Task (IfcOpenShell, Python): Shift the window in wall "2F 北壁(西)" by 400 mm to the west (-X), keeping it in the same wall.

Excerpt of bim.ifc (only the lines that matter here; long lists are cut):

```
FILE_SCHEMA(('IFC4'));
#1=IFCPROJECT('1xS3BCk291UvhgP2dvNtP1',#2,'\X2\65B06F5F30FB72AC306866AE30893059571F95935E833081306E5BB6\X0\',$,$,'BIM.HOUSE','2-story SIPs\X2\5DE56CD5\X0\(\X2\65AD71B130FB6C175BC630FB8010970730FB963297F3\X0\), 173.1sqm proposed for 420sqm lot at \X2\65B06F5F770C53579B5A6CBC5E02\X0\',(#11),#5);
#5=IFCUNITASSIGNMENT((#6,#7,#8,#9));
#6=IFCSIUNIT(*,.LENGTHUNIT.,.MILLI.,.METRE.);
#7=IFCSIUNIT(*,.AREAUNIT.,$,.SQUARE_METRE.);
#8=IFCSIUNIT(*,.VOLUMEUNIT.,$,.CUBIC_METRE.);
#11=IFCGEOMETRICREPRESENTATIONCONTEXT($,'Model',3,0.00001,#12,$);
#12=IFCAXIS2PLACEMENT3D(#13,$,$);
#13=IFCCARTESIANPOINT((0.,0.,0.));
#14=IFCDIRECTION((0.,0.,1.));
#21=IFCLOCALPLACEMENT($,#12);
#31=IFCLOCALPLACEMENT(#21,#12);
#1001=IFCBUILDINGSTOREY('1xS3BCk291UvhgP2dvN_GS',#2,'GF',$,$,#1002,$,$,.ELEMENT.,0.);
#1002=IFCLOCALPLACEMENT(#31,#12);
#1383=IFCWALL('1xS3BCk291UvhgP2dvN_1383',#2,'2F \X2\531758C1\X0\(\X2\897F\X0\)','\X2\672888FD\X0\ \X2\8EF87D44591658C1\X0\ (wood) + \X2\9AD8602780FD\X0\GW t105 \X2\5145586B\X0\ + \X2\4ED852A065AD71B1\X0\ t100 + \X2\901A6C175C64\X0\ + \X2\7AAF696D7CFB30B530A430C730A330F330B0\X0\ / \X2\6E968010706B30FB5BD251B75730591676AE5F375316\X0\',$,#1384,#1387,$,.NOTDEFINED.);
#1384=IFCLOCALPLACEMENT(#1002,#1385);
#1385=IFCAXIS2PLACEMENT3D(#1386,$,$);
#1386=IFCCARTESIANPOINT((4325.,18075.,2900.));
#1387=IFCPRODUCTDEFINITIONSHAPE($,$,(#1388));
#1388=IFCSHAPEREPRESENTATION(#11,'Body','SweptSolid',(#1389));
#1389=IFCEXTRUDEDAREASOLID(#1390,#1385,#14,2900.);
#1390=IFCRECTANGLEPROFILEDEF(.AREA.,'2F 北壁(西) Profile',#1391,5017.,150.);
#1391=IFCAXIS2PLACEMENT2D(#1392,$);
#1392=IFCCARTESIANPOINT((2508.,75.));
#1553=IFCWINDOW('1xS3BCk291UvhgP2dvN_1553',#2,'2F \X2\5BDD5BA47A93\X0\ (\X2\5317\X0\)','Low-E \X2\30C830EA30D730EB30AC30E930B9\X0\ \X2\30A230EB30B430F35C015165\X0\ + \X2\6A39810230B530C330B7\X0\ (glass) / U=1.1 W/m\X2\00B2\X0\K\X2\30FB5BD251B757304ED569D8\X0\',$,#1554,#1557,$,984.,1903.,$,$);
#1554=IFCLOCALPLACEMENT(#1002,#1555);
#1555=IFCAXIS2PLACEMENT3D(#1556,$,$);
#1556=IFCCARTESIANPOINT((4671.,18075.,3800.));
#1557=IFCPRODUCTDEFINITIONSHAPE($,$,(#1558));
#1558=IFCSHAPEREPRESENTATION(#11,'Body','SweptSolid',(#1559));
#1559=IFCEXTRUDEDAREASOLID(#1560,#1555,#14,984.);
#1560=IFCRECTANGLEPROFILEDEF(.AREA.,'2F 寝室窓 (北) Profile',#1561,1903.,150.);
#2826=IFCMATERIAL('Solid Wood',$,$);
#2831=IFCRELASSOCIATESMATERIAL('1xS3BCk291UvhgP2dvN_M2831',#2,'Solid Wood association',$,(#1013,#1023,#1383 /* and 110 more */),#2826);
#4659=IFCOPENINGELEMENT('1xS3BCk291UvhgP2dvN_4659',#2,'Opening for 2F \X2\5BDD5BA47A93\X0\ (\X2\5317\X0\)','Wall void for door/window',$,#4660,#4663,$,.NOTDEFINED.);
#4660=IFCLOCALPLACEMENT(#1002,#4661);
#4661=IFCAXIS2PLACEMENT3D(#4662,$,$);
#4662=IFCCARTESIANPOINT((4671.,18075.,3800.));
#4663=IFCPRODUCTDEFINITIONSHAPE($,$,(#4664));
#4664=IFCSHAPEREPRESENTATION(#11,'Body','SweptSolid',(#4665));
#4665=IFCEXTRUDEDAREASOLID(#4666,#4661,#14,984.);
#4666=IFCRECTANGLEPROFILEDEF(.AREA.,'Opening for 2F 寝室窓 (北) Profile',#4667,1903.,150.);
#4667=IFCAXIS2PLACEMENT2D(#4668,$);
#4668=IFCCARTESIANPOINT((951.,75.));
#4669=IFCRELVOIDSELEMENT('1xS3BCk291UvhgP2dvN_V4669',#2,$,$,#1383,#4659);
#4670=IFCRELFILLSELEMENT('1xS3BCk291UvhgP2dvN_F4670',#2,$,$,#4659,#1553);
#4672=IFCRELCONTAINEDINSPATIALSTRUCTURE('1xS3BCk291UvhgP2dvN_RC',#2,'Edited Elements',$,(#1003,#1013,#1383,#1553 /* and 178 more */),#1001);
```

```python
import ifcopenshell
import ifcopenshell.api.geometry
import ifcopenshell.util.placement

model = ifcopenshell.open("bim.ifc")

window = model.by_id(1553)
opening = window.FillsVoids[0].RelatingOpeningElement
wall = opening.VoidsElements[0].RelatingBuildingElement

wall_matrix = ifcopenshell.util.placement.get_local_placement(wall.ObjectPlacement)
shift = wall_matrix[:3, 0] * -400.0
before = ifcopenshell.util.placement.get_local_placement(window.ObjectPlacement)[:3, 3].copy()

# The window is not placed relative to its opening, so move both.
for product in (opening, window):
    matrix = ifcopenshell.util.placement.get_local_placement(product.ObjectPlacement)
    matrix[:3, 3] += shift
    ifcopenshell.api.geometry.edit_object_placement(model, product=product, matrix=matrix, is_si=False)

after = ifcopenshell.util.placement.get_local_placement(window.ObjectPlacement)[:3, 3]
print("window moved by", (after - before).round(3) + 0.0)

model.write("bim-out.ifc")
```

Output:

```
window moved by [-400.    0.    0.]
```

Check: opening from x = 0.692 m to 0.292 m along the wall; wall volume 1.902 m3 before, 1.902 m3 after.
